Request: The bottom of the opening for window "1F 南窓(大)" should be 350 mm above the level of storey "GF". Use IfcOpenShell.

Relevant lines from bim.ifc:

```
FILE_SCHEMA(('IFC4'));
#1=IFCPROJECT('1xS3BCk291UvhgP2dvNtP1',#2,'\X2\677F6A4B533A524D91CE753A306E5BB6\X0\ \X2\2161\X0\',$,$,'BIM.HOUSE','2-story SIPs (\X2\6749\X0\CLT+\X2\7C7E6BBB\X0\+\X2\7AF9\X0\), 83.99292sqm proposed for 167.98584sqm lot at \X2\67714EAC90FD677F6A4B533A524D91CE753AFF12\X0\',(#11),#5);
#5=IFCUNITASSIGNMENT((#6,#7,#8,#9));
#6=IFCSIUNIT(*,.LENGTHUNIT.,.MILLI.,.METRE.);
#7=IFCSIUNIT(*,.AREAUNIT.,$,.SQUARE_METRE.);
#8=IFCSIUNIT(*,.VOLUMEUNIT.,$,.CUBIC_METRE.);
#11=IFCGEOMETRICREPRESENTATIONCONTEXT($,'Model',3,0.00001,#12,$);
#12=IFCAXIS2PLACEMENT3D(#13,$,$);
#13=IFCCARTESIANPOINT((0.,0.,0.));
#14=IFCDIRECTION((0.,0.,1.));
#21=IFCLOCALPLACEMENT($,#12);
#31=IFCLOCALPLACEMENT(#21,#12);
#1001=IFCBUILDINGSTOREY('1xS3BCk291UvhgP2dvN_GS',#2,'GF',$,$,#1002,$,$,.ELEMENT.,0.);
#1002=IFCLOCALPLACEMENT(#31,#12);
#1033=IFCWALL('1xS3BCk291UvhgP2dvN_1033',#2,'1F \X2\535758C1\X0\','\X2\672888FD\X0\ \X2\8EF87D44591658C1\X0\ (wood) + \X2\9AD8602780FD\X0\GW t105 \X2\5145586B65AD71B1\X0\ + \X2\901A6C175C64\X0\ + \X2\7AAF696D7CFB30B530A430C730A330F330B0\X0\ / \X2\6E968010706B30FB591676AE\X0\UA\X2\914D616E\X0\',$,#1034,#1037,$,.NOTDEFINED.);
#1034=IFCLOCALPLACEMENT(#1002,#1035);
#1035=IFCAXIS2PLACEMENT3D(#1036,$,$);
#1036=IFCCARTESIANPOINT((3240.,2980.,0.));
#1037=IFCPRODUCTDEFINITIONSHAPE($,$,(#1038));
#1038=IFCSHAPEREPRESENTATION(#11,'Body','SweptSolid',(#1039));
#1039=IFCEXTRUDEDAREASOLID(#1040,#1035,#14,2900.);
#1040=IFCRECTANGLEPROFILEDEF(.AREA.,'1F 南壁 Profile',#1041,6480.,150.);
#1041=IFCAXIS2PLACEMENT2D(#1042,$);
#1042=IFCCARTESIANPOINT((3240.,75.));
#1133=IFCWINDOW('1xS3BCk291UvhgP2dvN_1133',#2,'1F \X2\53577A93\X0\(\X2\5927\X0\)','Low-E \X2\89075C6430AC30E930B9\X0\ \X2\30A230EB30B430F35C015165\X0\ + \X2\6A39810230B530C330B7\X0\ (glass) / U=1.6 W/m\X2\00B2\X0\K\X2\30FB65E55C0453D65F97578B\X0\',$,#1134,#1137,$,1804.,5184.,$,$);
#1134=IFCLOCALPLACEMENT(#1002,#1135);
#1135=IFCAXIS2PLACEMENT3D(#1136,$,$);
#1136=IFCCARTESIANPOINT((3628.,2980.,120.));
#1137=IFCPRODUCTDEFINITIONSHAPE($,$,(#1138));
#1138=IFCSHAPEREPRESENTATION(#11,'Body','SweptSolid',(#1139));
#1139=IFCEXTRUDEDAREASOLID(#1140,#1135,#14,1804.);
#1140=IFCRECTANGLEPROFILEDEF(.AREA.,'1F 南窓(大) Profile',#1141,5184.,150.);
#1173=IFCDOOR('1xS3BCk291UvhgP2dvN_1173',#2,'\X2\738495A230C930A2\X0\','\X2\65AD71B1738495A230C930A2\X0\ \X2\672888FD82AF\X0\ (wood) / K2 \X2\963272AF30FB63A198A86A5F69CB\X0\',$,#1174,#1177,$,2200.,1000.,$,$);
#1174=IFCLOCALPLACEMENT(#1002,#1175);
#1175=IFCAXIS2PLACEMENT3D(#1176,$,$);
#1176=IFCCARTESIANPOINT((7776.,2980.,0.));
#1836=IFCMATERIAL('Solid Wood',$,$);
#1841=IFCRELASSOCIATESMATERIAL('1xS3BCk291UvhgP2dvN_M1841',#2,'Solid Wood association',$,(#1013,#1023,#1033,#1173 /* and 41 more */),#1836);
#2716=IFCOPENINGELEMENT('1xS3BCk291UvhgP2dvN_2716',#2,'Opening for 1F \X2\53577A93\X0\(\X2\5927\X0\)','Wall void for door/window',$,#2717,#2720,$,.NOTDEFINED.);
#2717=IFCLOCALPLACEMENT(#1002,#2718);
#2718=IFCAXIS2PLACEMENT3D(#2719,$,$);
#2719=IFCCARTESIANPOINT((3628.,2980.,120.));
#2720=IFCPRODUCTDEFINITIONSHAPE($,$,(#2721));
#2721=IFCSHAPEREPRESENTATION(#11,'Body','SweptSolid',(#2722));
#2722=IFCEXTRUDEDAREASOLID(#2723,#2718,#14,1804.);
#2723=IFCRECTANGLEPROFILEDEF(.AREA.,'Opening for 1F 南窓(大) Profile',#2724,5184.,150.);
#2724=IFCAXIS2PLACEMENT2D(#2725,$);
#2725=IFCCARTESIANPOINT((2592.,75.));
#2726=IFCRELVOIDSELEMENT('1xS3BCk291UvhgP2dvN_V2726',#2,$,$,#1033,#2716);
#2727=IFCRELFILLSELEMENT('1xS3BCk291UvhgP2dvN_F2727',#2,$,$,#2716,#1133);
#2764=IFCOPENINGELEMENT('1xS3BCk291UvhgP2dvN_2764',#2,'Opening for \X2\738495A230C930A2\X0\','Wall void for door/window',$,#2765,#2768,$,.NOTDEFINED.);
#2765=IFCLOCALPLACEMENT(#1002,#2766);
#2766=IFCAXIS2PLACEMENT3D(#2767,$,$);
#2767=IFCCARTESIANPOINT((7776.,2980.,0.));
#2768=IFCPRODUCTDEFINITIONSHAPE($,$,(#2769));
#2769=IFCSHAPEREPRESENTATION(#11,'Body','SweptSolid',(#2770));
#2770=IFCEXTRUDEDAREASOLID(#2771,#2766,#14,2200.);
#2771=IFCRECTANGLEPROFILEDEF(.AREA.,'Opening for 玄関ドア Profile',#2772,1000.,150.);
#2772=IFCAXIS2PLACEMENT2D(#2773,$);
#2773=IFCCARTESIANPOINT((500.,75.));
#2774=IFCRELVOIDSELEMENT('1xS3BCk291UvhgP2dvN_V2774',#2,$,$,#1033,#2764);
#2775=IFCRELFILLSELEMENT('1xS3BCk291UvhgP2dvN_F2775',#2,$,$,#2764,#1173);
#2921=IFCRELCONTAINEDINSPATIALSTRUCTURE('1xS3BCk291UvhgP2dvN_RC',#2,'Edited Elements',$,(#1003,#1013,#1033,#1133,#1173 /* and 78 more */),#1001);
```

```python
import numpy as np
import ifcopenshell
import ifcopenshell.api.geometry
import ifcopenshell.geom
import ifcopenshell.util.element
import ifcopenshell.util.placement
import ifcopenshell.util.shape
import ifcopenshell.util.unit

model = ifcopenshell.open("bim.ifc")
unit_scale = ifcopenshell.util.unit.calculate_unit_scale(model)

window = model.by_id(1133)
opening = window.FillsVoids[0].RelatingOpeningElement
storey = ifcopenshell.util.element.get_container(window, ifc_class="IfcBuildingStorey")
level = ifcopenshell.util.placement.get_local_placement(storey.ObjectPlacement)[2, 3]

# The opening's origin need not be at the sill, so measure its lowest point.
shape = ifcopenshell.geom.create_shape(ifcopenshell.geom.settings(), opening)
bottom = ifcopenshell.util.shape.get_shape_bottom_elevation(shape, shape.geometry) / unit_scale
dz = level + 350.0 - bottom

shift = np.array([0.0, 0.0, dz])
# The window is not placed relative to its opening, so move both.
for product in (opening, window):
    matrix = ifcopenshell.util.placement.get_local_placement(product.ObjectPlacement)
    matrix[:3, 3] += shift
    ifcopenshell.api.geometry.edit_object_placement(model, product=product, matrix=matrix, is_si=False)

print(f"moved by {dz * unit_scale:+.3f} m")

model.write("bim-out.ifc")
```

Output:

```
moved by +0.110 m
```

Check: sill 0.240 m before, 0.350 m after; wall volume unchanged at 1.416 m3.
